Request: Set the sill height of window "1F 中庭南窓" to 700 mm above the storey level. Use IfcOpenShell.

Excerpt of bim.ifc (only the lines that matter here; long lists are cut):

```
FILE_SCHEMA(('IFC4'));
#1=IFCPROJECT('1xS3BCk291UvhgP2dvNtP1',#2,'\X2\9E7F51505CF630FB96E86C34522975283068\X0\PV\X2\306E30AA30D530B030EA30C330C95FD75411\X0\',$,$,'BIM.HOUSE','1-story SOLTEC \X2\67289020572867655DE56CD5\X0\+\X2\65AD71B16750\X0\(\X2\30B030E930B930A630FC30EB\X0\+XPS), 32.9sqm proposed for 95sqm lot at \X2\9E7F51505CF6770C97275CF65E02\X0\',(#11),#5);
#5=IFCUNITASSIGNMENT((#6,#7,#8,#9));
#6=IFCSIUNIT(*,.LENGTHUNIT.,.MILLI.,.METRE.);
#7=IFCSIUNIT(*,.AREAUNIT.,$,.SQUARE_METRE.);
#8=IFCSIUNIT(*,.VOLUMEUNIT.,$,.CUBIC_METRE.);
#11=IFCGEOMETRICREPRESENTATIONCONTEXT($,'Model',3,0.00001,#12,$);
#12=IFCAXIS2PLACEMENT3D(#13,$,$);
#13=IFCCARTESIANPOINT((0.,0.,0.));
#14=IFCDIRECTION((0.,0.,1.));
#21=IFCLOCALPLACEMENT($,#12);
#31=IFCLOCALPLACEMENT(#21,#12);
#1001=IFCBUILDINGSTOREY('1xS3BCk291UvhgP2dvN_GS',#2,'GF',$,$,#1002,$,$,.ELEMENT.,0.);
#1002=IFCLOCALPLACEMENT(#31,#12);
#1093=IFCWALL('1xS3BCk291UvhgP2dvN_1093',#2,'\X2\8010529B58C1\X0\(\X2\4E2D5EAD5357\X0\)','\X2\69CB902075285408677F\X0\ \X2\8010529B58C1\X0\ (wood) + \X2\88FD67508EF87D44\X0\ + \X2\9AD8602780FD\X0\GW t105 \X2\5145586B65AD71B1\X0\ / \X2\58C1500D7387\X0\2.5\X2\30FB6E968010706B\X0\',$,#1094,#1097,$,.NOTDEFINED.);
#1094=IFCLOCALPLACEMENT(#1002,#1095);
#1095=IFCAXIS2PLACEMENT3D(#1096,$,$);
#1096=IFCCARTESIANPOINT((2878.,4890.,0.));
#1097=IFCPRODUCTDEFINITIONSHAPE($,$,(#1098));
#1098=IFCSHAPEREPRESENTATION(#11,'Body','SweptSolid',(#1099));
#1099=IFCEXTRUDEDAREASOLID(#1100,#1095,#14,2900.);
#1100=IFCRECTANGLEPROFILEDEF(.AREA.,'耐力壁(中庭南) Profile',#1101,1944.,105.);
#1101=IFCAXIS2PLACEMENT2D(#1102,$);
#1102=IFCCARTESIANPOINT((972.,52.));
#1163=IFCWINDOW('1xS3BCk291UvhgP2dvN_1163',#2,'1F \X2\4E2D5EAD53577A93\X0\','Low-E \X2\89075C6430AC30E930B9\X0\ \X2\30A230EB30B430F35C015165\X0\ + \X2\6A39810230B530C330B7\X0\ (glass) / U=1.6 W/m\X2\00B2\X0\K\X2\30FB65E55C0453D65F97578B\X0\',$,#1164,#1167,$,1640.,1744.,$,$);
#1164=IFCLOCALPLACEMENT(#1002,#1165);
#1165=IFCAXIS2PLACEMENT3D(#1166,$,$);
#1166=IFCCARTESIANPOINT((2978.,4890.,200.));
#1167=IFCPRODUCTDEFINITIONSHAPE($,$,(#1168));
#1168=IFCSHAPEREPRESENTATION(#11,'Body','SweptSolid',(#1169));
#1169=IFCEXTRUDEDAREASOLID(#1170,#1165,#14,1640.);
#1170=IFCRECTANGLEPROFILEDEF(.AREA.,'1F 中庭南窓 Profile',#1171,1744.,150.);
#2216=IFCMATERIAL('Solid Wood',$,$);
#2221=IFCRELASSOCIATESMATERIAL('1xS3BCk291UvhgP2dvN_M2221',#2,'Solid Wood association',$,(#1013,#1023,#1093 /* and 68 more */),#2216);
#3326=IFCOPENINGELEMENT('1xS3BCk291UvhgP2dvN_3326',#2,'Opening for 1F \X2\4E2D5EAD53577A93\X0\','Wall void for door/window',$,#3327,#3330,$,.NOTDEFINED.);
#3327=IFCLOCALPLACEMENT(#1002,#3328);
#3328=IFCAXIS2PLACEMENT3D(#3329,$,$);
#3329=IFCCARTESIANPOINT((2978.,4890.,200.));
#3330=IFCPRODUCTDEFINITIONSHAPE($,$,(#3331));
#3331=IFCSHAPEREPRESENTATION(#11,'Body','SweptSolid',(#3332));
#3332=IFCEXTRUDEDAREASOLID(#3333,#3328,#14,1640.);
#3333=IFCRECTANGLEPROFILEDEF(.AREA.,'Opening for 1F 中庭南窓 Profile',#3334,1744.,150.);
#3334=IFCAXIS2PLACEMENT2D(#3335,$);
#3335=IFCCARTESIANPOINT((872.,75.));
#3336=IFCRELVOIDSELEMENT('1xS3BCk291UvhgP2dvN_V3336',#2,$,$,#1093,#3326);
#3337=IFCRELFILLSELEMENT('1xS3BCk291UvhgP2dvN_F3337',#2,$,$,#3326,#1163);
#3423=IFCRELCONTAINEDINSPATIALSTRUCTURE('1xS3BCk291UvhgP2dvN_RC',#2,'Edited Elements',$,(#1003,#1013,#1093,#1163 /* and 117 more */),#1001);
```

```python
import numpy as np
import ifcopenshell
import ifcopenshell.api.geometry
import ifcopenshell.geom
import ifcopenshell.util.element
import ifcopenshell.util.placement
import ifcopenshell.util.shape
import ifcopenshell.util.unit

model = ifcopenshell.open("bim.ifc")
unit_scale = ifcopenshell.util.unit.calculate_unit_scale(model)

window = model.by_guid("1xS3BCk291UvhgP2dvN_1163")
opening = window.FillsVoids[0].RelatingOpeningElement
storey = ifcopenshell.util.element.get_container(window, ifc_class="IfcBuildingStorey")
level = ifcopenshell.util.placement.get_local_placement(storey.ObjectPlacement)[2, 3]

# The opening's origin need not be at the sill, so measure its lowest point.
shape = ifcopenshell.geom.create_shape(ifcopenshell.geom.settings(), opening)
bottom = ifcopenshell.util.shape.get_shape_bottom_elevation(shape, shape.geometry) / unit_scale
dz = level + 700.0 - bottom

shift = np.array([0.0, 0.0, dz])
# The window is not placed relative to its opening, so move both.
for product in (opening, window):
    matrix = ifcopenshell.util.placement.get_local_placement(product.ObjectPlacement)
    matrix[:3, 3] += shift
    ifcopenshell.api.geometry.edit_object_placement(model, product=product, matrix=matrix, is_si=False)

print(f"moved by {dz * unit_scale:+.3f} m")

model.write("bim_rev.ifc")
```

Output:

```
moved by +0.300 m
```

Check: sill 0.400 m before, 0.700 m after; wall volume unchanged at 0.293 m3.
